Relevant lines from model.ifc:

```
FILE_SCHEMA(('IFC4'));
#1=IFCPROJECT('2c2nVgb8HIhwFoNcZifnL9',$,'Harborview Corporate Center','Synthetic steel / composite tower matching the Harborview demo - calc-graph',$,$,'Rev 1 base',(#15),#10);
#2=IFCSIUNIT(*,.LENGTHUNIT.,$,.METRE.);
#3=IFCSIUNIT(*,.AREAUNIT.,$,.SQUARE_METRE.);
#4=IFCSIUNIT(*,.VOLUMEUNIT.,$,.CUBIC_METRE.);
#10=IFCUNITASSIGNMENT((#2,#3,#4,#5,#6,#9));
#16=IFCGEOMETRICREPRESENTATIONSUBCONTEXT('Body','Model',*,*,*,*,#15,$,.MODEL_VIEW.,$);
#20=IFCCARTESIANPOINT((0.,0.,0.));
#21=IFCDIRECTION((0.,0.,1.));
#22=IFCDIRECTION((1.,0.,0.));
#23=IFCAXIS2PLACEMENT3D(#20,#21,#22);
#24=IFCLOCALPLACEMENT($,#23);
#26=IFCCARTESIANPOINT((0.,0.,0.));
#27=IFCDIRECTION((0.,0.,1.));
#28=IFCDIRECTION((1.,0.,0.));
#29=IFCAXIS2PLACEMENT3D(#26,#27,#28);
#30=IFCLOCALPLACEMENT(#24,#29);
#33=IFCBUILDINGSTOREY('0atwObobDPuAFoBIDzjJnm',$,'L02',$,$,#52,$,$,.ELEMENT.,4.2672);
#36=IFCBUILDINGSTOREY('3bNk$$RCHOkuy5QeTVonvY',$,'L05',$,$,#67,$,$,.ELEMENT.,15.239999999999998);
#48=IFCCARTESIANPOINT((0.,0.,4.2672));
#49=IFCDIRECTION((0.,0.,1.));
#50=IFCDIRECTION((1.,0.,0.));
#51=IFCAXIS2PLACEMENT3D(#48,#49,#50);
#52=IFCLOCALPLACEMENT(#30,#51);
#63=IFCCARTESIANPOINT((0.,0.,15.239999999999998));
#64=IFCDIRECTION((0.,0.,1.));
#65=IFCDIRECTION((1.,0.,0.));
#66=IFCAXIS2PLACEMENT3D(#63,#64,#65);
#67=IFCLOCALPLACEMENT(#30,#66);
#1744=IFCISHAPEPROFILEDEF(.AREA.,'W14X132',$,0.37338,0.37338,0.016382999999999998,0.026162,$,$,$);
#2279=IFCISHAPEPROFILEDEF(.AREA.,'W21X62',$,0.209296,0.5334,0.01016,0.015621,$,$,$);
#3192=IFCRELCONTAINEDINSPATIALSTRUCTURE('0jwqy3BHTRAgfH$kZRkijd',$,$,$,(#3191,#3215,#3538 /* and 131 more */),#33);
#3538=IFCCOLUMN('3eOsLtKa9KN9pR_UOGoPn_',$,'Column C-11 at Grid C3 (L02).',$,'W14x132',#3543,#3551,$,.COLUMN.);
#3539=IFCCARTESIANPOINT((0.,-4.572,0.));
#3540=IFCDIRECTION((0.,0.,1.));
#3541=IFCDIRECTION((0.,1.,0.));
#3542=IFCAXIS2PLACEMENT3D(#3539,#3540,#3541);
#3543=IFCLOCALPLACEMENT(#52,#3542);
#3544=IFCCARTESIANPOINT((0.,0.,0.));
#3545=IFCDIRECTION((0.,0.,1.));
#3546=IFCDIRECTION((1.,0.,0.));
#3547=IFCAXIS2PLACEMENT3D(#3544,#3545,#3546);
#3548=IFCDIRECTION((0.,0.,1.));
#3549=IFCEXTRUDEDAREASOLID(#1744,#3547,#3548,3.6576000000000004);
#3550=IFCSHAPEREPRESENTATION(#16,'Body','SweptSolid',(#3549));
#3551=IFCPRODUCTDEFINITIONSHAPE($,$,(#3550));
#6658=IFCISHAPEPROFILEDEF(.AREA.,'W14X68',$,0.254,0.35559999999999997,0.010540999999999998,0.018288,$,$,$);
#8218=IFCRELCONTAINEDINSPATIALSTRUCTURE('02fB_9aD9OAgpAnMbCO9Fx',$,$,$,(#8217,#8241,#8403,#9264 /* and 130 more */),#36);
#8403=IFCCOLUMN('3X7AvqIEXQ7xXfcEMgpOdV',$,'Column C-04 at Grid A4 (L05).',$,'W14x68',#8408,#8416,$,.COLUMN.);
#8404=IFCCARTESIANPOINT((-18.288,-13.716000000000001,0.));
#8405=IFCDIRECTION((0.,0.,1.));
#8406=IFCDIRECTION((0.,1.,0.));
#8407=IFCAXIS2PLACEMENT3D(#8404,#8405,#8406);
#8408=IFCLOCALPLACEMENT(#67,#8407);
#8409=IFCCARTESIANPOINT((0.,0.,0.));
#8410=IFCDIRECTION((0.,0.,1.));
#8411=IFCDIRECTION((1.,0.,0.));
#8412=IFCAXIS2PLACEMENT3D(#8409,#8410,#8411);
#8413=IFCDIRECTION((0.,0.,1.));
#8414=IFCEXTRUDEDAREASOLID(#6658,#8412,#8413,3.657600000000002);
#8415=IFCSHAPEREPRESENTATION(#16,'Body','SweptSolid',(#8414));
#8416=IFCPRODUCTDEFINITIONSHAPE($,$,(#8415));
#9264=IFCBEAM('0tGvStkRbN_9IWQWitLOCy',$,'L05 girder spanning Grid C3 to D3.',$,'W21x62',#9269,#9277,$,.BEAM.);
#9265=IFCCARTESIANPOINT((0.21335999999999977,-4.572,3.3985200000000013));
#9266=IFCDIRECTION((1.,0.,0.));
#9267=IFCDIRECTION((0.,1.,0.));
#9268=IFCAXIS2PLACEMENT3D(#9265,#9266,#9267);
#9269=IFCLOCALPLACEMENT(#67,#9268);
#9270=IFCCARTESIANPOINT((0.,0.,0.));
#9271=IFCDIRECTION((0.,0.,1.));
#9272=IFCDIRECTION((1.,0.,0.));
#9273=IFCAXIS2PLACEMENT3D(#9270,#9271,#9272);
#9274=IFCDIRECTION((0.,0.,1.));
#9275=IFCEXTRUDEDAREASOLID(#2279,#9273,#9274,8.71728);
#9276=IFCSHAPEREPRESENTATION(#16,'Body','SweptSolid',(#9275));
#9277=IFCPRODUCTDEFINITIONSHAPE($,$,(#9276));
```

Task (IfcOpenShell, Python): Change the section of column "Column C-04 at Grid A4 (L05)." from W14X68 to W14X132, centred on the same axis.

```python
import ifcopenshell
import ifcopenshell.util.element
import ifcopenshell.util.representation

model = ifcopenshell.open("model.ifc")

member = model.by_guid("3X7AvqIEXQ7xXfcEMgpOdV")
source = next(p for p in model.by_type("IfcIShapeProfileDef") if p.ProfileName == "W14X132")

body = ifcopenshell.util.representation.get_representation(member, "Model", "Body")
solid = body.Items[0]
old_profile = solid.SweptArea

# Copy the section's sizes but keep this member's own profile position.
profile = ifcopenshell.util.element.copy(model, source)
profile.Position = old_profile.Position
solid.SweptArea = profile
if not model.get_total_inverses(old_profile):
    ifcopenshell.util.element.remove_deep2(model, old_profile)

print(solid.SweptArea)

model.write("model-out.ifc")
```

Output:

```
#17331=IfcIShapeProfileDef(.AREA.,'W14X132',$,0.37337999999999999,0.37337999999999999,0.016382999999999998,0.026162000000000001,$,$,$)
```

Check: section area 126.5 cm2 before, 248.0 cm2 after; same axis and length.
